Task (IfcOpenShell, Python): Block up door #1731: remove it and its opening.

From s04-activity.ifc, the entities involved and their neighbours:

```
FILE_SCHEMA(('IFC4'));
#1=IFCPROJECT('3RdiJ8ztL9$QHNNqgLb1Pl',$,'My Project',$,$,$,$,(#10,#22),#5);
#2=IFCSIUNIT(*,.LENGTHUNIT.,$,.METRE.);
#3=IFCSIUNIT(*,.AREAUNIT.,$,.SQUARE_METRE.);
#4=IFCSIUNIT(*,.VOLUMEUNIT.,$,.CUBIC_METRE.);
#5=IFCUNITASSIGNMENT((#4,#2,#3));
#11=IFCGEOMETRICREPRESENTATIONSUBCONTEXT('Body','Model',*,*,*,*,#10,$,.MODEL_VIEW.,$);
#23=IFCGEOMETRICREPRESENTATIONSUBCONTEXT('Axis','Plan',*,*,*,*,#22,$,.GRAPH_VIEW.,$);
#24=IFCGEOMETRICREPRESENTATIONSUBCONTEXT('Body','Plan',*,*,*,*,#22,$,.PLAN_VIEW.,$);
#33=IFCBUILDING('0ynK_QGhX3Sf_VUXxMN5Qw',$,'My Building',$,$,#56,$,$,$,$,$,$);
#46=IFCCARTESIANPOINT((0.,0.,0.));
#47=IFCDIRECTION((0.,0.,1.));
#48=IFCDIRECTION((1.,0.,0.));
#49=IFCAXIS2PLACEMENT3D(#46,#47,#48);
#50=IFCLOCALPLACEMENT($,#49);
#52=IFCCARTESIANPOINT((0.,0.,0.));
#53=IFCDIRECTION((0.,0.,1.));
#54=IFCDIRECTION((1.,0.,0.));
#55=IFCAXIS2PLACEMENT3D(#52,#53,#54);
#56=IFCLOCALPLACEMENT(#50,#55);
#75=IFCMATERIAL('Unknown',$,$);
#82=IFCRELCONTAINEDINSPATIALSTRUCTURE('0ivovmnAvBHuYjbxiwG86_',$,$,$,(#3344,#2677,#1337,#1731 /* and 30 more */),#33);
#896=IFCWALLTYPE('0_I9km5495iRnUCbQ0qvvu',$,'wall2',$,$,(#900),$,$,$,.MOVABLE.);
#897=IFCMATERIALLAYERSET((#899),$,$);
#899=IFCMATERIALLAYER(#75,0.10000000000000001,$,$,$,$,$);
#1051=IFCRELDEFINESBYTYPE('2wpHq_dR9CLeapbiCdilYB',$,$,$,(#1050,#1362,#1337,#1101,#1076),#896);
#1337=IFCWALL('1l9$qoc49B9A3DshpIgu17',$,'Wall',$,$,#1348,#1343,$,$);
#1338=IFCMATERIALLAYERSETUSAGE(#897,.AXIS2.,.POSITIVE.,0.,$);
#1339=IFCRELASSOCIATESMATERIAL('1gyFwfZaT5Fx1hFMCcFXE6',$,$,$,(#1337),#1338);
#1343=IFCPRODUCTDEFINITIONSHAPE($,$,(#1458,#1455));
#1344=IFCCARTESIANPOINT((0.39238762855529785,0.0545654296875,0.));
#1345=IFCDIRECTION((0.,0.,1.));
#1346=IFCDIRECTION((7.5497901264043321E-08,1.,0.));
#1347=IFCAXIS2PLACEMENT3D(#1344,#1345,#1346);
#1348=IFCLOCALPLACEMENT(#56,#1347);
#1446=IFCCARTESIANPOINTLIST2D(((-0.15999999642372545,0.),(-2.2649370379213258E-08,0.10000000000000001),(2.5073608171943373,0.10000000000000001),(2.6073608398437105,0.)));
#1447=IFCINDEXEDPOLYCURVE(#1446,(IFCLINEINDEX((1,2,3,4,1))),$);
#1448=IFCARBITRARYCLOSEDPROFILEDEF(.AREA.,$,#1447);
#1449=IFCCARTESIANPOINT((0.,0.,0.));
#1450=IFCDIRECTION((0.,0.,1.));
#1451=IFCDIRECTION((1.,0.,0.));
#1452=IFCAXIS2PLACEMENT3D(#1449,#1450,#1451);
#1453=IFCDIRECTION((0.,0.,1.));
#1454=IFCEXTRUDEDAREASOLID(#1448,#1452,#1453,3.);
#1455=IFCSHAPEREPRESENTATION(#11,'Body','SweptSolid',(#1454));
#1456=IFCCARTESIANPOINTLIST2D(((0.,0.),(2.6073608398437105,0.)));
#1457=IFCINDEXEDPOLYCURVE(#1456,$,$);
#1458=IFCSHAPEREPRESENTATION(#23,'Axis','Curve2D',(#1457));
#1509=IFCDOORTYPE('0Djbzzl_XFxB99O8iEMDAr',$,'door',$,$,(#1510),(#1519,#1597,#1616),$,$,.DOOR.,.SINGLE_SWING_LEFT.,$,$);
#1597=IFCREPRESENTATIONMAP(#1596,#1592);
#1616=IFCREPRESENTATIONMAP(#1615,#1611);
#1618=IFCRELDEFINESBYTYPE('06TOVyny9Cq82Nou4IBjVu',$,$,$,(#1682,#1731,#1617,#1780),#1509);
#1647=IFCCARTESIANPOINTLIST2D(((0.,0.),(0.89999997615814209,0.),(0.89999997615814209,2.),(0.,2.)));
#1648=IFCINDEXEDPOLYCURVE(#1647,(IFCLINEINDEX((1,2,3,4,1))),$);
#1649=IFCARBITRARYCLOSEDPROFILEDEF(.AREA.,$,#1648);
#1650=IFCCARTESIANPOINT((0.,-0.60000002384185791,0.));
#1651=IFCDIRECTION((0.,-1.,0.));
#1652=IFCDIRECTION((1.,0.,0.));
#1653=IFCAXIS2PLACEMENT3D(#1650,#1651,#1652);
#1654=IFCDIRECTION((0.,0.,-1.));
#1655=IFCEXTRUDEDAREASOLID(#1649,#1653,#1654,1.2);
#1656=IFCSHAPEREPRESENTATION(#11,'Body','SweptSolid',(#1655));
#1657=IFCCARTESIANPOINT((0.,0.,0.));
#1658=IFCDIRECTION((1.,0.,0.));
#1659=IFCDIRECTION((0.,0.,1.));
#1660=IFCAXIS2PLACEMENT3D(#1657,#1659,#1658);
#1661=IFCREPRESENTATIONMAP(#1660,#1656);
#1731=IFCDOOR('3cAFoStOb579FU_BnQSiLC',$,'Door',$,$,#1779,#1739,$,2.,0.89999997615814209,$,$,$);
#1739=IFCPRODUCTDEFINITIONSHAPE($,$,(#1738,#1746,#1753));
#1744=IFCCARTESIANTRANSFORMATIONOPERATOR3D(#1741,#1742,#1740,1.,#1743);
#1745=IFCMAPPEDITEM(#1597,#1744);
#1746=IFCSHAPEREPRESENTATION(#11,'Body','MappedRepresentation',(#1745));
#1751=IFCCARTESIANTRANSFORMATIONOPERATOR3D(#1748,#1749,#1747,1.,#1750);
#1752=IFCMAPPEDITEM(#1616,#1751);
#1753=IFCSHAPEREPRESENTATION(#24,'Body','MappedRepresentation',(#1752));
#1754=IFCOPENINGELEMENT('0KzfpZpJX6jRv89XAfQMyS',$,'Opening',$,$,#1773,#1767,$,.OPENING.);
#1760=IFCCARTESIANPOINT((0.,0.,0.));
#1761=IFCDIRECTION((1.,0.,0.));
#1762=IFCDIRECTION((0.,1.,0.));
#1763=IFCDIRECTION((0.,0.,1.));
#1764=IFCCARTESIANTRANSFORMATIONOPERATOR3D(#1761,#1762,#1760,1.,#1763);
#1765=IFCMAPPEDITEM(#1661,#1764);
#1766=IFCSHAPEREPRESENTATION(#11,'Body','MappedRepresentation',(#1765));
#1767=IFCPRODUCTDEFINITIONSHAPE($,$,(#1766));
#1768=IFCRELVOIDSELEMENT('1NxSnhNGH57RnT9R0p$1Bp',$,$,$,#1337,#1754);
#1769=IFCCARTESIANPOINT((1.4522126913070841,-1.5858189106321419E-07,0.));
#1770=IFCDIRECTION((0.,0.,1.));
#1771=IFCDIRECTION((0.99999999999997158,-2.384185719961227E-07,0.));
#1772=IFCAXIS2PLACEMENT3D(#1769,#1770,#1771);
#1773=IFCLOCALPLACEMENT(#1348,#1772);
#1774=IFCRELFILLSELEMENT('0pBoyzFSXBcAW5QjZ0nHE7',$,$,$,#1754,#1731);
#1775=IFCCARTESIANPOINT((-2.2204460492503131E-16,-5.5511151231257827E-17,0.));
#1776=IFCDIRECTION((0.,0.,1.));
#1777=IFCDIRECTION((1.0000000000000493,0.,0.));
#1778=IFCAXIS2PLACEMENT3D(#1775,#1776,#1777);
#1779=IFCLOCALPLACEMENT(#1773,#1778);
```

```python
import ifcopenshell
import ifcopenshell.api.feature
import ifcopenshell.api.root
import ifcopenshell.geom
import ifcopenshell.util.shape

model = ifcopenshell.open("s04-activity.ifc")
settings = ifcopenshell.geom.settings()


def volume(element):
    """Net volume in cubic metres, openings subtracted."""
    shape = ifcopenshell.geom.create_shape(settings, element)
    return ifcopenshell.util.shape.get_volume(shape.geometry)


door = model.by_id(1731)
opening = door.FillsVoids[0].RelatingOpeningElement
wall = opening.VoidsElements[0].RelatingBuildingElement
before = volume(wall)

ifcopenshell.api.root.remove_product(model, product=door)
ifcopenshell.api.feature.remove_feature(model, feature=opening)

after = volume(wall)

print(f"wall volume {before:.3f} -> {after:.3f} m3")

model.write("s04-activity_updated.ifc")
```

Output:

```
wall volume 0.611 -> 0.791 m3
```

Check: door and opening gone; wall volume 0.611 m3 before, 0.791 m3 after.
